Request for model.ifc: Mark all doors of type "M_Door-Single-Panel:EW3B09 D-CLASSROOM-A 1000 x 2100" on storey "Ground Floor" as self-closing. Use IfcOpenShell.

First a look at what the model holds.

```python
import ifcopenshell
import ifcopenshell.util.element

model = ifcopenshell.open("model.ifc")
print(model.schema)
storey = next(s for s in model.by_type("IfcBuildingStorey") if s.Name == "Ground Floor")
doors = [e for e in ifcopenshell.util.element.get_decomposition(storey) if e.is_a("IfcDoor")]
seen = {}
for e in doors:
    element_type = ifcopenshell.util.element.get_type(e)
    key = (element_type.Name if element_type != e and element_type else None, ifcopenshell.util.element.get_pset(e, "Pset_DoorCommon", "SelfClosing"))
    seen[key] = seen.get(key, 0) + 1
for (name, value), count in sorted(seen.items(), key=str):
    print(count, "x", name, "|", value)
```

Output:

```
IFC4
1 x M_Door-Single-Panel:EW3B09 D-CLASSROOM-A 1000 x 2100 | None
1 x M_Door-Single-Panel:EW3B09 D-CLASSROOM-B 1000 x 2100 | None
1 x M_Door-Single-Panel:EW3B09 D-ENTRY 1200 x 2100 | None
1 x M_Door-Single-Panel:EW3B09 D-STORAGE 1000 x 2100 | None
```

```python
import ifcopenshell
import ifcopenshell.api.pset
import ifcopenshell.util.element

model = ifcopenshell.open("model.ifc")

storey = next(s for s in model.by_type("IfcBuildingStorey") if s.Name == "Ground Floor")
doors = [e for e in ifcopenshell.util.element.get_decomposition(storey) if e.is_a("IfcDoor")]

count = 0
for e in doors:
    element_type = ifcopenshell.util.element.get_type(e)
    if element_type in (None, e) or element_type.Name != "M_Door-Single-Panel:EW3B09 D-CLASSROOM-A 1000 x 2100":
        continue
    # add_pset returns the element's existing set when there is one.
    pset = ifcopenshell.api.pset.add_pset(model, product=e, name="Pset_DoorCommon")
    ifcopenshell.api.pset.edit_pset(model, pset=pset, properties={"SelfClosing": True})
    count += 1

print(count, "doors updated")

model.write("model_edited.ifc")
```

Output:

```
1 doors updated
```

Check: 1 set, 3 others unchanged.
